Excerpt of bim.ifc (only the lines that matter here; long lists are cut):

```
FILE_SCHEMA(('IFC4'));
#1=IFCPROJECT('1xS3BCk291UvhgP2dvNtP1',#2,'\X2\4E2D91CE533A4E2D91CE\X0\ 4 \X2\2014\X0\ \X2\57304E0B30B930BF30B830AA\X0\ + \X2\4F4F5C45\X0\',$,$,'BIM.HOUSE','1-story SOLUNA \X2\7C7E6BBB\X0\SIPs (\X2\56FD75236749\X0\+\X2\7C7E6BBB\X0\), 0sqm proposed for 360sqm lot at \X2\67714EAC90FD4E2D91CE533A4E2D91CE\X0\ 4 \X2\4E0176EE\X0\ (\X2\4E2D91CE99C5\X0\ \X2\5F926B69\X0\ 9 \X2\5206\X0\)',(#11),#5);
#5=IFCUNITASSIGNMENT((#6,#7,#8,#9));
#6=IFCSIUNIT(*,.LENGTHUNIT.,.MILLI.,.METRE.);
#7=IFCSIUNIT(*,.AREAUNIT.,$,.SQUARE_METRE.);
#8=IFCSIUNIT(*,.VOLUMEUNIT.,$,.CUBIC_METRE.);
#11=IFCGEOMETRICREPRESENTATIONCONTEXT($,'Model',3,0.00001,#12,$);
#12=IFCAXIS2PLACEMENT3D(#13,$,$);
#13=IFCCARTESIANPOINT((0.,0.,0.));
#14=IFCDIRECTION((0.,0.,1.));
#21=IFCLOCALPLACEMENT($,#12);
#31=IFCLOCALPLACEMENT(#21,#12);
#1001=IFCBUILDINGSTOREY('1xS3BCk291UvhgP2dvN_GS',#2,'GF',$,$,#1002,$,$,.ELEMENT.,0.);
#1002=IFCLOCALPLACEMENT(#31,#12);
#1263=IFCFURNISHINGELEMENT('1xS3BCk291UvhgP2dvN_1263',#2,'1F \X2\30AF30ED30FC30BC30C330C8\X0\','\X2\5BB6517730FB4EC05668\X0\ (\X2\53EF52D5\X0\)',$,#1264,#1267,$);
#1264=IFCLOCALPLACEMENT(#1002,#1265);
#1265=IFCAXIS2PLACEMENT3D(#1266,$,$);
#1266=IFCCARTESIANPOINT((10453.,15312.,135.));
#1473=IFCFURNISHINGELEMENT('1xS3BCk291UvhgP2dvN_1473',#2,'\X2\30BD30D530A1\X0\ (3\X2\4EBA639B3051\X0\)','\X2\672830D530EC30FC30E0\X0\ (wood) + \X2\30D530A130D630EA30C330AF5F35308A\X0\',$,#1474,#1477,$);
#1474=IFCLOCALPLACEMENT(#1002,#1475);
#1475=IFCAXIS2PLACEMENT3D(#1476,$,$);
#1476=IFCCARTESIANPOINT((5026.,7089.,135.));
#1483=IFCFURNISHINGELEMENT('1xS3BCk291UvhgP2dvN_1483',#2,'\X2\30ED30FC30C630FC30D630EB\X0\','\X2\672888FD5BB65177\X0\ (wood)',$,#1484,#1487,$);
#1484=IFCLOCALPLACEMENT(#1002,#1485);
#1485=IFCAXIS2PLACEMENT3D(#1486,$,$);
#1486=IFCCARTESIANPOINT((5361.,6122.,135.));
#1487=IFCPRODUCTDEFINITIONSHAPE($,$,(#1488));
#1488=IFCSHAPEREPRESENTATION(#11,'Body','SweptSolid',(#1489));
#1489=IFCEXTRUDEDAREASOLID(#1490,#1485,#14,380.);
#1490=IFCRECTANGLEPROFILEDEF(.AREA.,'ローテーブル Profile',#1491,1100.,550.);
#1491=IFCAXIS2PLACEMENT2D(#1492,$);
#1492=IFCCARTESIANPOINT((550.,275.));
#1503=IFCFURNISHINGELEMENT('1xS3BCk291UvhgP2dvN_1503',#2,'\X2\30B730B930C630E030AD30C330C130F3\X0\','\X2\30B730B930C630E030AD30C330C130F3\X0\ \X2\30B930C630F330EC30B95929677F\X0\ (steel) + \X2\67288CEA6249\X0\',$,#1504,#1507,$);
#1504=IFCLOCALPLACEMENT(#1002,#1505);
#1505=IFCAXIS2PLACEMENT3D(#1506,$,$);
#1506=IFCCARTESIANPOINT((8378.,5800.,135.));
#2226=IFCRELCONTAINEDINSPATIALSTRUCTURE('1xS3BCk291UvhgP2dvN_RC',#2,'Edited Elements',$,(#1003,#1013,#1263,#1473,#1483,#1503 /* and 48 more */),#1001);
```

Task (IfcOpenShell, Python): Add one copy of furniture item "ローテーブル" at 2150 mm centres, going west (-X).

```python
import numpy as np
import ifcopenshell
import ifcopenshell.api.geometry
import ifcopenshell.api.root
import ifcopenshell.util.element
import ifcopenshell.util.placement

model = ifcopenshell.open("bim.ifc")


def reuse_history(source, copy):
    """copy_class also copies each property set's owner history, people and application; keep the originals."""
    for rel in copy.IsDefinedBy:
        if rel.is_a("IfcRelDefinesByProperties") and (history := rel.RelatingPropertyDefinition.OwnerHistory):
            rel.RelatingPropertyDefinition.OwnerHistory = source.OwnerHistory
            ifcopenshell.util.element.remove_deep2(model, history)


source = model.by_guid("1xS3BCk291UvhgP2dvN_1483")
base = ifcopenshell.util.placement.get_local_placement(source.ObjectPlacement)
step = np.array([-1.0, 0.0, 0.0]) * 2150.0

for i in range(1, 2):
    copy = ifcopenshell.api.root.copy_class(model, product=source)
    copy.Representation = ifcopenshell.util.element.copy_deep(
        model, source.Representation, exclude=["IfcGeometricRepresentationContext", "IfcRepresentationMap"]
    )
    reuse_history(source, copy)
    matrix = base.copy()
    matrix[:3, 3] += i * step
    print("added at", matrix[:3, 3].round(3) + 0.0)
    ifcopenshell.api.geometry.edit_object_placement(model, product=copy, matrix=matrix, is_si=False)

model.write("bim_edited.ifc")
```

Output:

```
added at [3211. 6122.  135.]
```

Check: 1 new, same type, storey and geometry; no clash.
